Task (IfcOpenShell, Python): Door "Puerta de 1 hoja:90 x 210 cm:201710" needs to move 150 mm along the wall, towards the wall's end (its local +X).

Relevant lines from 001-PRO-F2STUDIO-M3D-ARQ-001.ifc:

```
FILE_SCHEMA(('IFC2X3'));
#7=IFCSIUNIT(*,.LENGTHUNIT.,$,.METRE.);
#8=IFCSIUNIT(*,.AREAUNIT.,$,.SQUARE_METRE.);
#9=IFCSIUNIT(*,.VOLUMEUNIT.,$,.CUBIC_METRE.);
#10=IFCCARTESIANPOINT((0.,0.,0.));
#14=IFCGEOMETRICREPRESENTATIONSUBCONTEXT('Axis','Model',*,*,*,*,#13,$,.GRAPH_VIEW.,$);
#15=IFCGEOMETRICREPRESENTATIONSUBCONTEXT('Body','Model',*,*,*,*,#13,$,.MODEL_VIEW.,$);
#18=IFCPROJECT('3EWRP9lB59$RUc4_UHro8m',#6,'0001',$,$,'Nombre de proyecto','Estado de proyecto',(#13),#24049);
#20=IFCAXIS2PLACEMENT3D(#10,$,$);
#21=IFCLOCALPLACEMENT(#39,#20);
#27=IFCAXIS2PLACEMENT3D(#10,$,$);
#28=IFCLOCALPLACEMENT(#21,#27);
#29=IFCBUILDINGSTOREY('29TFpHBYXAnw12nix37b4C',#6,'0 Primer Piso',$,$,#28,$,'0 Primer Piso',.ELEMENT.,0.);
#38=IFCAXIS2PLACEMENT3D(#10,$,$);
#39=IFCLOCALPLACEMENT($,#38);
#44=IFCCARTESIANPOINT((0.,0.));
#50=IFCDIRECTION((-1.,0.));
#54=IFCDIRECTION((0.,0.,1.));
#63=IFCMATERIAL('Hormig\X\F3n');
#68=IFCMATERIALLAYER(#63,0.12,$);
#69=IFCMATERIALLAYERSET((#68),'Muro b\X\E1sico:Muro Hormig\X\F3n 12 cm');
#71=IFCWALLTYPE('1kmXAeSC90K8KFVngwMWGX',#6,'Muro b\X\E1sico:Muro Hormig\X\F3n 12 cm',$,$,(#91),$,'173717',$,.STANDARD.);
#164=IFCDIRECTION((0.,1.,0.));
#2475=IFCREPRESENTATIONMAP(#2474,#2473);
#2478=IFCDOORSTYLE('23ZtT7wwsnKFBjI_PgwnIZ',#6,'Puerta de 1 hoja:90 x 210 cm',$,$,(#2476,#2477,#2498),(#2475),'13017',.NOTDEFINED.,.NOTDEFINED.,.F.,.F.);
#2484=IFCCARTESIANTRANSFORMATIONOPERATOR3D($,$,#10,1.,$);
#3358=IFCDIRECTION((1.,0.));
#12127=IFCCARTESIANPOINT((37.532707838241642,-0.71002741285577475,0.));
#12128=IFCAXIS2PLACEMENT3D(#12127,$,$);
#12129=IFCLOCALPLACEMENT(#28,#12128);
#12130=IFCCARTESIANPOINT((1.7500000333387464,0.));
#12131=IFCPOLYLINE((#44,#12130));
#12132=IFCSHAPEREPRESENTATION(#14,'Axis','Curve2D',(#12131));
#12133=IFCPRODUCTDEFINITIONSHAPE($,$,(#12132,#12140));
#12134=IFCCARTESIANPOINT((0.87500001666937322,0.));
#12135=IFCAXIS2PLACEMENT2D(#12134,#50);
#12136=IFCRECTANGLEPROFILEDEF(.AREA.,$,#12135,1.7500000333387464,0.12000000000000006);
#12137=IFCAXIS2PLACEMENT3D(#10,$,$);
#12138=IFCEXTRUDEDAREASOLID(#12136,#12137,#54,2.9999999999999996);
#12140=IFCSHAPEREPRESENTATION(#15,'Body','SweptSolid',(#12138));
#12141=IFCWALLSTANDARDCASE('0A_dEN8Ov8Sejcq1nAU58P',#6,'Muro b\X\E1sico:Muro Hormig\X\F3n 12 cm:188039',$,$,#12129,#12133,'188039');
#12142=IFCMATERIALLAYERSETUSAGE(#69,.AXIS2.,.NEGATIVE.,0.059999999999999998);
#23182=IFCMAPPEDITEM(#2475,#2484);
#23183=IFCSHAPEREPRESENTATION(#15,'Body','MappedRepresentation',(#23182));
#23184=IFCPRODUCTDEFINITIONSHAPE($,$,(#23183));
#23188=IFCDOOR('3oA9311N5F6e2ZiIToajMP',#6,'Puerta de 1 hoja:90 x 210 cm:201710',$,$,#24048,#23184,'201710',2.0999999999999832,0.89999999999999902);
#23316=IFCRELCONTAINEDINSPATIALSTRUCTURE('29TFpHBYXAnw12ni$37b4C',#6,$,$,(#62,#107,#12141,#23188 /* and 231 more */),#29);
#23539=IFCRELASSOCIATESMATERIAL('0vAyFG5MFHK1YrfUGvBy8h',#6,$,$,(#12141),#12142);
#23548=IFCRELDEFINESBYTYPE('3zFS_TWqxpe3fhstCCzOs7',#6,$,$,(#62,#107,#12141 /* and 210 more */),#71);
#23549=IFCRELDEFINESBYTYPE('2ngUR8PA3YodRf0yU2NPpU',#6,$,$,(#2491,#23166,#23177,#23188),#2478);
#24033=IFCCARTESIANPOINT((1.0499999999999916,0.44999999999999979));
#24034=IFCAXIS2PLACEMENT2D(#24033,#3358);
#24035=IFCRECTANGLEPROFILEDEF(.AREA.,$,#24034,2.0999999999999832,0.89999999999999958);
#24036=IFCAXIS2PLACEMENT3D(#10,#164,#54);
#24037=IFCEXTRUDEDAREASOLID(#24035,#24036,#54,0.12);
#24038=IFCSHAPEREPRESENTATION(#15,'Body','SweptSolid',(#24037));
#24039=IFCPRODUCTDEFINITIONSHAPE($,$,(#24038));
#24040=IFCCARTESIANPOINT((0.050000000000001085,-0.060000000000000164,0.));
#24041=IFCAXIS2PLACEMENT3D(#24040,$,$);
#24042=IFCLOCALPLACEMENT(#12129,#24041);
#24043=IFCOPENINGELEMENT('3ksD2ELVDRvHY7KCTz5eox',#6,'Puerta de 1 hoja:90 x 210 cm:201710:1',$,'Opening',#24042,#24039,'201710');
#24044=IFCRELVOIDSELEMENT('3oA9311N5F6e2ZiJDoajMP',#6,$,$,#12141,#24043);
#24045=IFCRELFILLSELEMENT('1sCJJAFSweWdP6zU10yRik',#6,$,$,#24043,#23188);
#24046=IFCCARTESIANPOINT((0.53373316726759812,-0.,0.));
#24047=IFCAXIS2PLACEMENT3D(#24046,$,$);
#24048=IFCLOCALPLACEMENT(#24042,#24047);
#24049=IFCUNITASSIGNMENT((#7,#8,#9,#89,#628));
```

```python
import ifcopenshell
import ifcopenshell.api.geometry
import ifcopenshell.util.placement

model = ifcopenshell.open("001-PRO-F2STUDIO-M3D-ARQ-001.ifc")

door = model.by_id(23188)
opening = door.FillsVoids[0].RelatingOpeningElement
wall = opening.VoidsElements[0].RelatingBuildingElement

wall_matrix = ifcopenshell.util.placement.get_local_placement(wall.ObjectPlacement)
shift = wall_matrix[:3, 0] * 0.15
before = ifcopenshell.util.placement.get_local_placement(door.ObjectPlacement)[:3, 3].copy()

# The door is placed relative to its opening, so it follows when the opening moves.
matrix = ifcopenshell.util.placement.get_local_placement(opening.ObjectPlacement)
matrix[:3, 3] += shift
ifcopenshell.api.geometry.edit_object_placement(
    model, product=opening, matrix=matrix, is_si=False, should_transform_children=True
)

after = ifcopenshell.util.placement.get_local_placement(door.ObjectPlacement)[:3, 3]
print("door moved by", (after - before).round(3) + 0.0)

model.write("001-PRO-F2STUDIO-M3D-ARQ-001_v2.ifc")
```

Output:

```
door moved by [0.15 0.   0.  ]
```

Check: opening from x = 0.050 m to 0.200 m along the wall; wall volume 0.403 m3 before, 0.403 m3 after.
